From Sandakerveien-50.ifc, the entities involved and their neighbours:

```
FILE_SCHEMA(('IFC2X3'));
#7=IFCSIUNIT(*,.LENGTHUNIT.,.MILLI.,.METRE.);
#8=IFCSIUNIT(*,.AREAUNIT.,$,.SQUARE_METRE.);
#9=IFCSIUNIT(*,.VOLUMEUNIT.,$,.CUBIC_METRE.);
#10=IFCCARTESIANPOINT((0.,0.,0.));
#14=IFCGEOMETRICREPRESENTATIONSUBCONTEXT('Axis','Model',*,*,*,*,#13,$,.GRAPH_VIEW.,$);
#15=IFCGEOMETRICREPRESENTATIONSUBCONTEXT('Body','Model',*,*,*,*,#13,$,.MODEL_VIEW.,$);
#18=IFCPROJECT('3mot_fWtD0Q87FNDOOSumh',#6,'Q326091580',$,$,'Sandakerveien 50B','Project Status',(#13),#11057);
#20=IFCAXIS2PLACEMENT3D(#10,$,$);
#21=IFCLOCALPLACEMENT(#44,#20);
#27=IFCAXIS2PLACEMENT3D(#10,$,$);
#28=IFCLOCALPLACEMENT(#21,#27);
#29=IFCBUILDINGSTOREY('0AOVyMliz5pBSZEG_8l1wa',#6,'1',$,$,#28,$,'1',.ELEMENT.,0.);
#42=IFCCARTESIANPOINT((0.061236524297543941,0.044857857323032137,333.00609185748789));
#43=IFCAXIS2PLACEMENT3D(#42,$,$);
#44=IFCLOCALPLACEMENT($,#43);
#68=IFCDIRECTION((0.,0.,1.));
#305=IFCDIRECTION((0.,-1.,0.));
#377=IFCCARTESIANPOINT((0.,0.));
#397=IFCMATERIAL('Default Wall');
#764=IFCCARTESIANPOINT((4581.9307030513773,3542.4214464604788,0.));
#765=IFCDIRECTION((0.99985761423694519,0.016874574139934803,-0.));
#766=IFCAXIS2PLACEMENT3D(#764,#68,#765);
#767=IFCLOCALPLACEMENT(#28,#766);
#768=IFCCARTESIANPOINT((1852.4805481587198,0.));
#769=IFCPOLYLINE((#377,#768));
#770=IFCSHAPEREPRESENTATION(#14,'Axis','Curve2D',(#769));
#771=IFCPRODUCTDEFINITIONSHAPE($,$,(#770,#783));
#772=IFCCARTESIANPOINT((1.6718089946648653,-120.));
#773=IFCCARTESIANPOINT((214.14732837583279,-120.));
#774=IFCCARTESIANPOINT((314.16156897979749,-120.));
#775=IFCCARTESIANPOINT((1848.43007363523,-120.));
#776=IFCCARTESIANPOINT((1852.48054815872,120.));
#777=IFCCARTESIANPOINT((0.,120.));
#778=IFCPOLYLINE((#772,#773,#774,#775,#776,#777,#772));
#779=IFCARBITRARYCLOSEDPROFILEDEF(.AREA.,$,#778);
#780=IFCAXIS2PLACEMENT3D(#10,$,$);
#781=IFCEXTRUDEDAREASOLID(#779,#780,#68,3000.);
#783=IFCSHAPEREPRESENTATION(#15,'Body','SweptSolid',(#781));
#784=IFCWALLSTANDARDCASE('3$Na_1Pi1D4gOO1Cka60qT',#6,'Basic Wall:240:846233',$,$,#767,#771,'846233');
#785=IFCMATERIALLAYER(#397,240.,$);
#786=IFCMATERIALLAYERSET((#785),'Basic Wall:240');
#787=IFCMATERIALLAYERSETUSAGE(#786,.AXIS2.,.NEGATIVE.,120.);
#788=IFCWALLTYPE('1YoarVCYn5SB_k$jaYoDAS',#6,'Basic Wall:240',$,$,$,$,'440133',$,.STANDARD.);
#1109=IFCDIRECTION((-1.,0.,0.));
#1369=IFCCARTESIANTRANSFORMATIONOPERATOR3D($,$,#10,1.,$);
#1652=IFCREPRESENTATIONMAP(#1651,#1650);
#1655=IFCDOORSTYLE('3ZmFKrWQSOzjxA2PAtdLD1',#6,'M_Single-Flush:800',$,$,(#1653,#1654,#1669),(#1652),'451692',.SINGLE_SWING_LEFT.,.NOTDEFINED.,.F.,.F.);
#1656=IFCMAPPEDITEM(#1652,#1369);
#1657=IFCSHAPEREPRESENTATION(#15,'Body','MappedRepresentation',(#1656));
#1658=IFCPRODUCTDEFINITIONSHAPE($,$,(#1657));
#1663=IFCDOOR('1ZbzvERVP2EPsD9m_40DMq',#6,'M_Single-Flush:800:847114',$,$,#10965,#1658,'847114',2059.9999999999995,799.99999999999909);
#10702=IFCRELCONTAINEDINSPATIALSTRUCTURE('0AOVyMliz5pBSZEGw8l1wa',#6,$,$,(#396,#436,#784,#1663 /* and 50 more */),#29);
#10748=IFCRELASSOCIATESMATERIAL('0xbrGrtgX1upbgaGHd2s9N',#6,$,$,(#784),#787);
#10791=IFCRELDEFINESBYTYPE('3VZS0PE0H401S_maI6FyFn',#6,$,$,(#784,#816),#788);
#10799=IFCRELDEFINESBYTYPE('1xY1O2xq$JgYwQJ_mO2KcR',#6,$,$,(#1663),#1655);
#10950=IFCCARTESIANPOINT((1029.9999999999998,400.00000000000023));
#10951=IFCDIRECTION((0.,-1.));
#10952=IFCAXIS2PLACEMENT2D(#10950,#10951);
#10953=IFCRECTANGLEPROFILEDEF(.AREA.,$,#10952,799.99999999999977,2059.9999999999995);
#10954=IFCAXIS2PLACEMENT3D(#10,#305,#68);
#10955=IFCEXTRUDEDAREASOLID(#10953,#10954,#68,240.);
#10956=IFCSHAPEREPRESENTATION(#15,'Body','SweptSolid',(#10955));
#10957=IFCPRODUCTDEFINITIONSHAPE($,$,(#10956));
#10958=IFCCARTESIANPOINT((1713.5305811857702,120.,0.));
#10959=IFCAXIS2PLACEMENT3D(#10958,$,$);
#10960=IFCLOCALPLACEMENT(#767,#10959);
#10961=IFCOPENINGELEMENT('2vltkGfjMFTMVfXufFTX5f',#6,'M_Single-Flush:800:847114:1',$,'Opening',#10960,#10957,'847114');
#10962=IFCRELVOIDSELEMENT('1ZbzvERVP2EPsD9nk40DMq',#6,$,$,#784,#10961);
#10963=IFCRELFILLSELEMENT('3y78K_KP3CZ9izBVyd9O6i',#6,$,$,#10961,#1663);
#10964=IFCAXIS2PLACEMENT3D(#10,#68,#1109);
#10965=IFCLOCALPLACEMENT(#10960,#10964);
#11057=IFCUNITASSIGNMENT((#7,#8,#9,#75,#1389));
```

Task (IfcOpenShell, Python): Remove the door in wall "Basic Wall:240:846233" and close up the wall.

```python
import ifcopenshell
import ifcopenshell.api.feature
import ifcopenshell.api.root
import ifcopenshell.geom
import ifcopenshell.util.shape

model = ifcopenshell.open("Sandakerveien-50.ifc")
settings = ifcopenshell.geom.settings()


def volume(element):
    """Net volume in cubic metres, openings subtracted."""
    shape = ifcopenshell.geom.create_shape(settings, element)
    return ifcopenshell.util.shape.get_volume(shape.geometry)


door = model.by_id(1663)
opening = door.FillsVoids[0].RelatingOpeningElement
wall = opening.VoidsElements[0].RelatingBuildingElement
before = volume(wall)

ifcopenshell.api.root.remove_product(model, product=door)
ifcopenshell.api.feature.remove_feature(model, feature=opening)

after = volume(wall)

print(f"wall volume {before:.3f} -> {after:.3f} m3")

model.write("Sandakerveien-50_updated.ifc")
```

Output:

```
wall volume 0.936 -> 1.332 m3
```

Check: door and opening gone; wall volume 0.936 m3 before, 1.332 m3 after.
